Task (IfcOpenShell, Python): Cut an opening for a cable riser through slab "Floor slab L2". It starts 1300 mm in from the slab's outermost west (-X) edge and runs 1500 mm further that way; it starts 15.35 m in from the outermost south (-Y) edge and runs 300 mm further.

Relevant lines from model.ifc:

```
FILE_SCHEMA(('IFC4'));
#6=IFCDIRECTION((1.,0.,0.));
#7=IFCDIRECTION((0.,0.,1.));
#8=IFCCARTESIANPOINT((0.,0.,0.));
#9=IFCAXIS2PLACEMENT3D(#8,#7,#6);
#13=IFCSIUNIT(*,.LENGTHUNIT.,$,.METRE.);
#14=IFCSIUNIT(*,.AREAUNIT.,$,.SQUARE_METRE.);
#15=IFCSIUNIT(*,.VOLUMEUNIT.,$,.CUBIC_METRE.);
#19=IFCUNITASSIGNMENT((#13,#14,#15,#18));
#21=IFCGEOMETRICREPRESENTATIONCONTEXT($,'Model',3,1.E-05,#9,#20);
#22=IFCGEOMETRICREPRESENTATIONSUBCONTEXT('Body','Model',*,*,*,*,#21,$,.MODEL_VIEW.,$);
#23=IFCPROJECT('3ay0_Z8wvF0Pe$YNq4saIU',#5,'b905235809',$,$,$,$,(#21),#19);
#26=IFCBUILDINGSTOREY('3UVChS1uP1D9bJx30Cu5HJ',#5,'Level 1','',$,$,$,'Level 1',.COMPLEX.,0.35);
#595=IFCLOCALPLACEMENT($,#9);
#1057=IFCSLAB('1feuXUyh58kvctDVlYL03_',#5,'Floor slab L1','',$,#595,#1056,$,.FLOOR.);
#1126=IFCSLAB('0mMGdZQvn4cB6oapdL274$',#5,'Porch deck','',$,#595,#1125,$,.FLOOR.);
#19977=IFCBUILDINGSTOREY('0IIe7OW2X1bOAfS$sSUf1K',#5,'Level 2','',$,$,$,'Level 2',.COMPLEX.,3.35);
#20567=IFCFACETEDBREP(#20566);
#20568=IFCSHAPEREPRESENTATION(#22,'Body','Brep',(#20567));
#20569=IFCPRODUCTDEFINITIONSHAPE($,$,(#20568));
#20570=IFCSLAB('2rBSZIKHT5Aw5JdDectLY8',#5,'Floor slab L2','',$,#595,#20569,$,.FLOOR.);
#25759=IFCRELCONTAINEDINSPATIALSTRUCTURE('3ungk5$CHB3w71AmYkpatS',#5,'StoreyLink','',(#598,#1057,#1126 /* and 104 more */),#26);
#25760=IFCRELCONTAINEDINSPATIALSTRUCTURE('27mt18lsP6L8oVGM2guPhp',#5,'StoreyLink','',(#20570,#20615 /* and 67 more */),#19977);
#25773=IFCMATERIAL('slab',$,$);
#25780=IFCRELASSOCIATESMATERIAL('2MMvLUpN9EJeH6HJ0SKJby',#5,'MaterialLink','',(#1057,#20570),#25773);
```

```python
import numpy as np
import ifcopenshell
import ifcopenshell.api.feature
import ifcopenshell.api.geometry
import ifcopenshell.api.root
import ifcopenshell.geom
import ifcopenshell.util.placement
import ifcopenshell.util.representation
import ifcopenshell.util.shape
import ifcopenshell.util.unit

model = ifcopenshell.open("model.ifc")
unit_scale = ifcopenshell.util.unit.calculate_unit_scale(model)
settings = ifcopenshell.geom.settings()


def volume(element):
    """Net volume in cubic metres, openings subtracted."""
    shape = ifcopenshell.geom.create_shape(settings, element)
    return ifcopenshell.util.shape.get_volume(shape.geometry)


slab = model.by_guid("2rBSZIKHT5Aw5JdDectLY8")
before = volume(slab)

# Extent in the slab's own axes, in metres. The edges named are its -X and -Y sides.
slab_shape = ifcopenshell.geom.create_shape(settings, slab)
vertices = ifcopenshell.util.shape.get_vertices(slab_shape.geometry)
x_min, y_min, bottom = vertices.min(axis=0)
top = vertices[:, 2].max()

opening = ifcopenshell.api.root.create_entity(model, ifc_class="IfcOpeningElement", name="Cable riser opening", predefined_type="OPENING")
context = ifcopenshell.util.representation.get_context(model, "Model", "Body", "MODEL_VIEW")
width, depth = 1.5, 0.3
outline = [(0.0, 0.0), (width, 0.0), (width, depth), (0.0, depth), (0.0, 0.0)]
# Overshoot both faces by 50 mm so the cut is clean.
shape = ifcopenshell.api.geometry.add_slab_representation(
    model, context=context, depth=top - bottom + 0.1, polyline=outline
)
ifcopenshell.api.geometry.assign_representation(model, product=opening, representation=shape)

matrix = ifcopenshell.util.placement.get_local_placement(slab.ObjectPlacement)
matrix[:, 3] = matrix @ np.append(np.array([x_min + 1.3, y_min + 15.35, bottom - 0.05]) / unit_scale, 1.0)
ifcopenshell.api.geometry.edit_object_placement(model, product=opening, matrix=matrix, is_si=False)
ifcopenshell.api.feature.add_feature(model, feature=opening, element=slab)

after = volume(slab)

print(f"slab volume {before:.3f} -> {after:.3f} m3")

model.write("model_v2.ifc")
```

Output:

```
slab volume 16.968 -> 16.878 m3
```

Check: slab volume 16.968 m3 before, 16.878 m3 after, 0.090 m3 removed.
